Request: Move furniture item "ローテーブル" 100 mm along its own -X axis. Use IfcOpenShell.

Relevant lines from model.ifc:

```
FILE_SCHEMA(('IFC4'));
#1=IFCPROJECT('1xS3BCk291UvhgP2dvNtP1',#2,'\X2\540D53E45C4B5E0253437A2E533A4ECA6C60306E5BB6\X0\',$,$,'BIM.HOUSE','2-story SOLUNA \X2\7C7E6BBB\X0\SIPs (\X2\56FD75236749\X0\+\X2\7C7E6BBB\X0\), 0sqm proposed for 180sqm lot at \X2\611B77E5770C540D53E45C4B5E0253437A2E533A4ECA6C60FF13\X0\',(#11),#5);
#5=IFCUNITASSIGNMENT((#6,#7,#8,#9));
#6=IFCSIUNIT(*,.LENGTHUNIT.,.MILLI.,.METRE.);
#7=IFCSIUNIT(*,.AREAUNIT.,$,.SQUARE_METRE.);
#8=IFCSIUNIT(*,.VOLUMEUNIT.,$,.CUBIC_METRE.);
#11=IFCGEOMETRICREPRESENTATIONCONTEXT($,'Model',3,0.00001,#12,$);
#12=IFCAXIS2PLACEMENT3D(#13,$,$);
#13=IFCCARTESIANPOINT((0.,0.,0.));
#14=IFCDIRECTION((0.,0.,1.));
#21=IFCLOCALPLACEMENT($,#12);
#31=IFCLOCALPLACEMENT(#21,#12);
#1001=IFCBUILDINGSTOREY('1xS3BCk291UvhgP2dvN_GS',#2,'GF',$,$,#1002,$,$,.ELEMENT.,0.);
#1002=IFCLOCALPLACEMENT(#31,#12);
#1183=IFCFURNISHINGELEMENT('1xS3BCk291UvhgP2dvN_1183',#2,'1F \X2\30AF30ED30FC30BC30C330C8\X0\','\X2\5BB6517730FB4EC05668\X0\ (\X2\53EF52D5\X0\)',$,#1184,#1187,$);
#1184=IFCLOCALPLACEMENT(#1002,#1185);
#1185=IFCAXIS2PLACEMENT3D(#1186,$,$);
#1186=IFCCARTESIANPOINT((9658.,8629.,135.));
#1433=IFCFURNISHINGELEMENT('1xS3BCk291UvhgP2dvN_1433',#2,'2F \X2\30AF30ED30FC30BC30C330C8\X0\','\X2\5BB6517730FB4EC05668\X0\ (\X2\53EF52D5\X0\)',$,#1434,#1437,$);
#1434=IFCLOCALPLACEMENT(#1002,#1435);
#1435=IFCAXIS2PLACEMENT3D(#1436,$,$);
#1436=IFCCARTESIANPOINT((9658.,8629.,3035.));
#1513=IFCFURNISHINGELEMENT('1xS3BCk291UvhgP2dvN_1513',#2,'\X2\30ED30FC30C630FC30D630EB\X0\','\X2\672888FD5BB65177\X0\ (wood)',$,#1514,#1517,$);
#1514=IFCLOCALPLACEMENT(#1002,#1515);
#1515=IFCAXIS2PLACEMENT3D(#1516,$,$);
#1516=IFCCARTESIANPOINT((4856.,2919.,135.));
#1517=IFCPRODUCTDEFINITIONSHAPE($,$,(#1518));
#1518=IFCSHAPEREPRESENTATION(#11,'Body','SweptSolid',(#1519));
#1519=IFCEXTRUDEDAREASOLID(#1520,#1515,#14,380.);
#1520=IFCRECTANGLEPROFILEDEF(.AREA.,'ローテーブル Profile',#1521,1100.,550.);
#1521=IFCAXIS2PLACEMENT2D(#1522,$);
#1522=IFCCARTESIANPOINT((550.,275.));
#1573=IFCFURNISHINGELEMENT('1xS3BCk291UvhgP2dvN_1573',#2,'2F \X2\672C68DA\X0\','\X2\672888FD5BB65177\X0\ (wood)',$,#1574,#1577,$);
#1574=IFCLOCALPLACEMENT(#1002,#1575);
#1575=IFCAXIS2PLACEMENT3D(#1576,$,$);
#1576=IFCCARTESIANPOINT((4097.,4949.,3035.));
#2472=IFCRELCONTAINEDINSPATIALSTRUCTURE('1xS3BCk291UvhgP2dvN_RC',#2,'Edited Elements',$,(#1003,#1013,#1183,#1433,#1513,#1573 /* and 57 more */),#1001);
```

```python
import ifcopenshell
import ifcopenshell.api.geometry
import ifcopenshell.util.placement

model = ifcopenshell.open("model.ifc")

item = model.by_id(1513)
matrix = ifcopenshell.util.placement.get_local_placement(item.ObjectPlacement)
matrix[:3, 3] -= matrix[:3, 0] * 100.0
ifcopenshell.api.geometry.edit_object_placement(model, product=item, matrix=matrix, is_si=False)

print(ifcopenshell.util.placement.get_local_placement(item.ObjectPlacement).round(3) + 0.0)

model.write("model_updated.ifc")
```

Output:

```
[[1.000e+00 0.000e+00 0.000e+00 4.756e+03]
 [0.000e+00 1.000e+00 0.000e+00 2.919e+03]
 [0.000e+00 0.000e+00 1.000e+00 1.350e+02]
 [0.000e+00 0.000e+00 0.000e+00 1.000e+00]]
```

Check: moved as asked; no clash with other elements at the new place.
